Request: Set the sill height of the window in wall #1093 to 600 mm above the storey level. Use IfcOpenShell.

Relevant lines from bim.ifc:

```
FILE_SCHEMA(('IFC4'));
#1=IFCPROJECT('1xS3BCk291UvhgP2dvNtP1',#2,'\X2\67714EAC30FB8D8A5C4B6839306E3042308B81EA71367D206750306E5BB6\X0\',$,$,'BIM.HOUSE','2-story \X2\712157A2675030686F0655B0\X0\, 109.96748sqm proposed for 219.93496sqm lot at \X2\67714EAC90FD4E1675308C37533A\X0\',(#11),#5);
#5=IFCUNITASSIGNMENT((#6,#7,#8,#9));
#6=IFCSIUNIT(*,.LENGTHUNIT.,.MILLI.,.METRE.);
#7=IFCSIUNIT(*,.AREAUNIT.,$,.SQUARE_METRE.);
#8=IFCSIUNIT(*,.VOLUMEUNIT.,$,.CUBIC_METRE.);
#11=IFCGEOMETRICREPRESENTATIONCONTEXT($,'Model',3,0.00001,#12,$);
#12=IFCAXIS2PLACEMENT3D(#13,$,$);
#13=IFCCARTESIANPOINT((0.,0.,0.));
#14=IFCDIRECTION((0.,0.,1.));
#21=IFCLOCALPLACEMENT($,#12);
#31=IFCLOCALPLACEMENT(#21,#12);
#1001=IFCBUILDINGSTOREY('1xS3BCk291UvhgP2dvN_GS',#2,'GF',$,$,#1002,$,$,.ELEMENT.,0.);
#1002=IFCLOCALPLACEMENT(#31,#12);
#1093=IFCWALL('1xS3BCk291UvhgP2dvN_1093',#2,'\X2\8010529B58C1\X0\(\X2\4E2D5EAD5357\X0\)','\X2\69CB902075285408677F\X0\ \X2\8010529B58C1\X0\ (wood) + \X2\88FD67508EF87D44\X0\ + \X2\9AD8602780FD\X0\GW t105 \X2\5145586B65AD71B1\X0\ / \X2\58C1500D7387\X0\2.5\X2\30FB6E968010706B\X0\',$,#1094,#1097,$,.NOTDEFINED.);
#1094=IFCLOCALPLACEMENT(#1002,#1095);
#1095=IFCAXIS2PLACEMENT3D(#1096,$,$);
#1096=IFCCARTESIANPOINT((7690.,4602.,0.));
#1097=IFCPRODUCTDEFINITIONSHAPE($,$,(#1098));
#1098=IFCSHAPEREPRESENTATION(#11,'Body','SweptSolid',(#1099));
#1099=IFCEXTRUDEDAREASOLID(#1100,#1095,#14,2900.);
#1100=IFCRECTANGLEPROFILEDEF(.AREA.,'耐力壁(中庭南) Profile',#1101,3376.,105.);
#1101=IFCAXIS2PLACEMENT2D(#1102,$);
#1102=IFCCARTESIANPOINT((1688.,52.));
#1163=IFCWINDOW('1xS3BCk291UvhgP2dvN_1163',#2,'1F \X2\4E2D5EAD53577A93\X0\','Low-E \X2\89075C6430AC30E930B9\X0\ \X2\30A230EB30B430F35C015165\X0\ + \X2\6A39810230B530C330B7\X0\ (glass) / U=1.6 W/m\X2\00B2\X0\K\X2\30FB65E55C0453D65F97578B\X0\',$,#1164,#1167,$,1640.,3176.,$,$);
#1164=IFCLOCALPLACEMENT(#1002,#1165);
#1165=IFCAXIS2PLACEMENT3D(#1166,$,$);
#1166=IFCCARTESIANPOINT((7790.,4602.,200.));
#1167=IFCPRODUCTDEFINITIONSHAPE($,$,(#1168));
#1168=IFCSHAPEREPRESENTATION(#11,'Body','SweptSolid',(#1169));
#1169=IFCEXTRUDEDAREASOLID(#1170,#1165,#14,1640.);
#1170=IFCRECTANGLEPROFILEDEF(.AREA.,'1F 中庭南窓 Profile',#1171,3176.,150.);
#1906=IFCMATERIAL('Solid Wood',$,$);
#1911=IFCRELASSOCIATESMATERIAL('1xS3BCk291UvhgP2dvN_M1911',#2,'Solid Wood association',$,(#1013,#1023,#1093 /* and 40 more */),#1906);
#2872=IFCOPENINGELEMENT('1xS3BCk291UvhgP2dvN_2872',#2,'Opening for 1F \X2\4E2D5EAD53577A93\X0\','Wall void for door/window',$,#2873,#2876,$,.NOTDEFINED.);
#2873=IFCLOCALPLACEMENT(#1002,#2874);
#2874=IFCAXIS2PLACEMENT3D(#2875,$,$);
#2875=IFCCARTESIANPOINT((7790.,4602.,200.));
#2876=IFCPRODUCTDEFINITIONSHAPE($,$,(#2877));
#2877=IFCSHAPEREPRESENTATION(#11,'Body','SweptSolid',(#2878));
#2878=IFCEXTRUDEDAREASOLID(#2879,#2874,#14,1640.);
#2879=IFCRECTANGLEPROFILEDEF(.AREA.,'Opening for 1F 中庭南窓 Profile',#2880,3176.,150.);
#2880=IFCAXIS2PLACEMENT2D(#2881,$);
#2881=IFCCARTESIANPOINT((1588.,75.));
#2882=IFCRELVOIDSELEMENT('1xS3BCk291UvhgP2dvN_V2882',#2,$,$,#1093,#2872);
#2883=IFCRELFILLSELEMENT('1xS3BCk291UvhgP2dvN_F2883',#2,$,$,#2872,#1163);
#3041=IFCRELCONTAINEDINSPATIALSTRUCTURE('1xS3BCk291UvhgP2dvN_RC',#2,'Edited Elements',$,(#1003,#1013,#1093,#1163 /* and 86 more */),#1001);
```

```python
import numpy as np
import ifcopenshell
import ifcopenshell.api.geometry
import ifcopenshell.geom
import ifcopenshell.util.element
import ifcopenshell.util.placement
import ifcopenshell.util.shape
import ifcopenshell.util.unit

model = ifcopenshell.open("bim.ifc")
unit_scale = ifcopenshell.util.unit.calculate_unit_scale(model)

window = model.by_guid("1xS3BCk291UvhgP2dvN_1163")
opening = window.FillsVoids[0].RelatingOpeningElement
storey = ifcopenshell.util.element.get_container(window, ifc_class="IfcBuildingStorey")
level = ifcopenshell.util.placement.get_local_placement(storey.ObjectPlacement)[2, 3]

# The opening's origin need not be at the sill, so measure its lowest point.
shape = ifcopenshell.geom.create_shape(ifcopenshell.geom.settings(), opening)
bottom = ifcopenshell.util.shape.get_shape_bottom_elevation(shape, shape.geometry) / unit_scale
dz = level + 0.6 / unit_scale - bottom

shift = np.array([0.0, 0.0, dz])
# The window is not placed relative to its opening, so move both.
for product in (opening, window):
    matrix = ifcopenshell.util.placement.get_local_placement(product.ObjectPlacement)
    matrix[:3, 3] += shift
    ifcopenshell.api.geometry.edit_object_placement(model, product=product, matrix=matrix, is_si=False)

print(f"moved by {dz * unit_scale:+.3f} m")

model.write("bim_edited.ifc")
```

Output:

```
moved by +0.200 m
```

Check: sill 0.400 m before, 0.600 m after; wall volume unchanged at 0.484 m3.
